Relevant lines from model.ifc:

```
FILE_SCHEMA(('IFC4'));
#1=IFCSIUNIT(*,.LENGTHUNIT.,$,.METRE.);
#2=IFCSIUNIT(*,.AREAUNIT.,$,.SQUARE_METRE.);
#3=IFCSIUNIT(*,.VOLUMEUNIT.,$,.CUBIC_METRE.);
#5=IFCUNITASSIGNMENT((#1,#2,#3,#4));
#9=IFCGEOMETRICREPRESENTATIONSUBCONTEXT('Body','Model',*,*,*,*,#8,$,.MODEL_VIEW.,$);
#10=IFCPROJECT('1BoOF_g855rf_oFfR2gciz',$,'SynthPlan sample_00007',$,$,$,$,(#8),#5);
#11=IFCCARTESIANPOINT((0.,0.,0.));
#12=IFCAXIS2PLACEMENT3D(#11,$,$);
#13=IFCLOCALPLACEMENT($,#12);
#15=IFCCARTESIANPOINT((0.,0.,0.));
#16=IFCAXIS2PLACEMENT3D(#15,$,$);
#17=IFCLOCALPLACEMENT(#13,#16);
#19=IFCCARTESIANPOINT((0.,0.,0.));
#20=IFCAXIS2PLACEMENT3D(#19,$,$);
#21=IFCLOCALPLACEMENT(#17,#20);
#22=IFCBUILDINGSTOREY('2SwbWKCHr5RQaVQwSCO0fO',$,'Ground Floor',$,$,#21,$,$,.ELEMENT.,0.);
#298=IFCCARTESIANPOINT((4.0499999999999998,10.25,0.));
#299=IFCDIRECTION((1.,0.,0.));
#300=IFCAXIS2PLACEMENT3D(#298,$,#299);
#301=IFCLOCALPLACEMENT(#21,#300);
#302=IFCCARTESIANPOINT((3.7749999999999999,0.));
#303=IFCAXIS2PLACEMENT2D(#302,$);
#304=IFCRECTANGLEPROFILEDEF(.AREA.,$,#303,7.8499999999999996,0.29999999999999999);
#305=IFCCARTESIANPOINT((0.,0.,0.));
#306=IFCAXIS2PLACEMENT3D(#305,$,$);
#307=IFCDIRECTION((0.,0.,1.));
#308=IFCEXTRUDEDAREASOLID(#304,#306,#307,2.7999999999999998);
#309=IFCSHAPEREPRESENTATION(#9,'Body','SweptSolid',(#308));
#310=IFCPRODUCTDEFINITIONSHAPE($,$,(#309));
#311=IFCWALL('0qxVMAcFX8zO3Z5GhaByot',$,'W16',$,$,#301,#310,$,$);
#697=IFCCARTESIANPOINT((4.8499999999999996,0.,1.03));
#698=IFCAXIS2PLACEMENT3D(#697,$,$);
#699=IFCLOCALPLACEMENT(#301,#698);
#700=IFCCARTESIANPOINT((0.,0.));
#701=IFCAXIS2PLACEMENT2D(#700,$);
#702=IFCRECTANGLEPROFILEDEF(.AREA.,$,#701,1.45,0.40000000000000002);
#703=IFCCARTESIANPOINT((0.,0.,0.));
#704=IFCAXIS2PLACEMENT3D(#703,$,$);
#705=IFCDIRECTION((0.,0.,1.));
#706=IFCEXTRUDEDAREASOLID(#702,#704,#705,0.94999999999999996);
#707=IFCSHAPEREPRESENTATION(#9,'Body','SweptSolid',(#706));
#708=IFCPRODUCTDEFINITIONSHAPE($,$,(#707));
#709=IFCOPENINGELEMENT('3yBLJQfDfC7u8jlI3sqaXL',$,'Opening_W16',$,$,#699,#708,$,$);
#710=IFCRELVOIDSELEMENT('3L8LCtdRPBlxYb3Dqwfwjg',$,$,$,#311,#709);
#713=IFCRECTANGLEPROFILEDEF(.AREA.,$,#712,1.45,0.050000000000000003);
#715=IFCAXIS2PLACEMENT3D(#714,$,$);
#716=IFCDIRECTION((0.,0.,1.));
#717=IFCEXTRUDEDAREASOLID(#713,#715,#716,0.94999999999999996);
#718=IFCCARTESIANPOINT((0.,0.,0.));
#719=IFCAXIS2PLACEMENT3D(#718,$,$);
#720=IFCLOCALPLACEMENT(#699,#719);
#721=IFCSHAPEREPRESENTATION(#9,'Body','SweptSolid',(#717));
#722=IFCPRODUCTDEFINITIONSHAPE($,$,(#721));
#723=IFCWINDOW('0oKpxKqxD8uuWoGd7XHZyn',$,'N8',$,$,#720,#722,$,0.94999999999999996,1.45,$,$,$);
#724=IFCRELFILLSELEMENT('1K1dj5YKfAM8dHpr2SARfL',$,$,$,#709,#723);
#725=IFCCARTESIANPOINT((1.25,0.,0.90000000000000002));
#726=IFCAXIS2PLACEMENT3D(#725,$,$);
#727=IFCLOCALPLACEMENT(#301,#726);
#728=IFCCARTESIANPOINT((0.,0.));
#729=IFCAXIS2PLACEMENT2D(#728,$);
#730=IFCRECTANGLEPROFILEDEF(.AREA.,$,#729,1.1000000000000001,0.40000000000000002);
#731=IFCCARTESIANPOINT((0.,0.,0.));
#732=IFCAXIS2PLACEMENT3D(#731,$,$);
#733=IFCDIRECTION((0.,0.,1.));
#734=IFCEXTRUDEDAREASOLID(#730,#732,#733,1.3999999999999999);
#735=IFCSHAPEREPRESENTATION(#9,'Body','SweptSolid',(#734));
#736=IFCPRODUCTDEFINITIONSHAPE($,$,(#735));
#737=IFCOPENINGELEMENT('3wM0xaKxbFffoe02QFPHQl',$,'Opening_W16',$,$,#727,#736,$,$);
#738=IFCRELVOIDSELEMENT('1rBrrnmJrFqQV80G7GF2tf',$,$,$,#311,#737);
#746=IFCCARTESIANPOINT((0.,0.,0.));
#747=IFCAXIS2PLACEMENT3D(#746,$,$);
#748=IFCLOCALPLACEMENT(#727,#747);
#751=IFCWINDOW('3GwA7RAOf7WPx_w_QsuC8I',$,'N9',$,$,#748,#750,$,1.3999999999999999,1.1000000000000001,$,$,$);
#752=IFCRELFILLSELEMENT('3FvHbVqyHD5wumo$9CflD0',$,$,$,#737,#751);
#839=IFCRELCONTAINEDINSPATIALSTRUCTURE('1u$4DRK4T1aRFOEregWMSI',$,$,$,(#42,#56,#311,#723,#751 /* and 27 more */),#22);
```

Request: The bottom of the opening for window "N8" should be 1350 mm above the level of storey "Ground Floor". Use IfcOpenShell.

```python
import numpy as np
import ifcopenshell
import ifcopenshell.api.geometry
import ifcopenshell.geom
import ifcopenshell.util.element
import ifcopenshell.util.placement
import ifcopenshell.util.shape
import ifcopenshell.util.unit

model = ifcopenshell.open("model.ifc")
unit_scale = ifcopenshell.util.unit.calculate_unit_scale(model)

window = model.by_guid("0oKpxKqxD8uuWoGd7XHZyn")
opening = window.FillsVoids[0].RelatingOpeningElement
storey = ifcopenshell.util.element.get_container(window, ifc_class="IfcBuildingStorey")
level = ifcopenshell.util.placement.get_local_placement(storey.ObjectPlacement)[2, 3]

# The opening's origin need not be at the sill, so measure its lowest point.
shape = ifcopenshell.geom.create_shape(ifcopenshell.geom.settings(), opening)
bottom = ifcopenshell.util.shape.get_shape_bottom_elevation(shape, shape.geometry) / unit_scale
dz = level + 1.35 / unit_scale - bottom

shift = np.array([0.0, 0.0, dz])
# The window is placed relative to its opening, so it follows when the opening moves.
matrix = ifcopenshell.util.placement.get_local_placement(opening.ObjectPlacement)
matrix[:3, 3] += shift
ifcopenshell.api.geometry.edit_object_placement(
    model, product=opening, matrix=matrix, is_si=False, should_transform_children=True
)

print(f"moved by {dz * unit_scale:+.3f} m")

model.write("model_edited.ifc")
```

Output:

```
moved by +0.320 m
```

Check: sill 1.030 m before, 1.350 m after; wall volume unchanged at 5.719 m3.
